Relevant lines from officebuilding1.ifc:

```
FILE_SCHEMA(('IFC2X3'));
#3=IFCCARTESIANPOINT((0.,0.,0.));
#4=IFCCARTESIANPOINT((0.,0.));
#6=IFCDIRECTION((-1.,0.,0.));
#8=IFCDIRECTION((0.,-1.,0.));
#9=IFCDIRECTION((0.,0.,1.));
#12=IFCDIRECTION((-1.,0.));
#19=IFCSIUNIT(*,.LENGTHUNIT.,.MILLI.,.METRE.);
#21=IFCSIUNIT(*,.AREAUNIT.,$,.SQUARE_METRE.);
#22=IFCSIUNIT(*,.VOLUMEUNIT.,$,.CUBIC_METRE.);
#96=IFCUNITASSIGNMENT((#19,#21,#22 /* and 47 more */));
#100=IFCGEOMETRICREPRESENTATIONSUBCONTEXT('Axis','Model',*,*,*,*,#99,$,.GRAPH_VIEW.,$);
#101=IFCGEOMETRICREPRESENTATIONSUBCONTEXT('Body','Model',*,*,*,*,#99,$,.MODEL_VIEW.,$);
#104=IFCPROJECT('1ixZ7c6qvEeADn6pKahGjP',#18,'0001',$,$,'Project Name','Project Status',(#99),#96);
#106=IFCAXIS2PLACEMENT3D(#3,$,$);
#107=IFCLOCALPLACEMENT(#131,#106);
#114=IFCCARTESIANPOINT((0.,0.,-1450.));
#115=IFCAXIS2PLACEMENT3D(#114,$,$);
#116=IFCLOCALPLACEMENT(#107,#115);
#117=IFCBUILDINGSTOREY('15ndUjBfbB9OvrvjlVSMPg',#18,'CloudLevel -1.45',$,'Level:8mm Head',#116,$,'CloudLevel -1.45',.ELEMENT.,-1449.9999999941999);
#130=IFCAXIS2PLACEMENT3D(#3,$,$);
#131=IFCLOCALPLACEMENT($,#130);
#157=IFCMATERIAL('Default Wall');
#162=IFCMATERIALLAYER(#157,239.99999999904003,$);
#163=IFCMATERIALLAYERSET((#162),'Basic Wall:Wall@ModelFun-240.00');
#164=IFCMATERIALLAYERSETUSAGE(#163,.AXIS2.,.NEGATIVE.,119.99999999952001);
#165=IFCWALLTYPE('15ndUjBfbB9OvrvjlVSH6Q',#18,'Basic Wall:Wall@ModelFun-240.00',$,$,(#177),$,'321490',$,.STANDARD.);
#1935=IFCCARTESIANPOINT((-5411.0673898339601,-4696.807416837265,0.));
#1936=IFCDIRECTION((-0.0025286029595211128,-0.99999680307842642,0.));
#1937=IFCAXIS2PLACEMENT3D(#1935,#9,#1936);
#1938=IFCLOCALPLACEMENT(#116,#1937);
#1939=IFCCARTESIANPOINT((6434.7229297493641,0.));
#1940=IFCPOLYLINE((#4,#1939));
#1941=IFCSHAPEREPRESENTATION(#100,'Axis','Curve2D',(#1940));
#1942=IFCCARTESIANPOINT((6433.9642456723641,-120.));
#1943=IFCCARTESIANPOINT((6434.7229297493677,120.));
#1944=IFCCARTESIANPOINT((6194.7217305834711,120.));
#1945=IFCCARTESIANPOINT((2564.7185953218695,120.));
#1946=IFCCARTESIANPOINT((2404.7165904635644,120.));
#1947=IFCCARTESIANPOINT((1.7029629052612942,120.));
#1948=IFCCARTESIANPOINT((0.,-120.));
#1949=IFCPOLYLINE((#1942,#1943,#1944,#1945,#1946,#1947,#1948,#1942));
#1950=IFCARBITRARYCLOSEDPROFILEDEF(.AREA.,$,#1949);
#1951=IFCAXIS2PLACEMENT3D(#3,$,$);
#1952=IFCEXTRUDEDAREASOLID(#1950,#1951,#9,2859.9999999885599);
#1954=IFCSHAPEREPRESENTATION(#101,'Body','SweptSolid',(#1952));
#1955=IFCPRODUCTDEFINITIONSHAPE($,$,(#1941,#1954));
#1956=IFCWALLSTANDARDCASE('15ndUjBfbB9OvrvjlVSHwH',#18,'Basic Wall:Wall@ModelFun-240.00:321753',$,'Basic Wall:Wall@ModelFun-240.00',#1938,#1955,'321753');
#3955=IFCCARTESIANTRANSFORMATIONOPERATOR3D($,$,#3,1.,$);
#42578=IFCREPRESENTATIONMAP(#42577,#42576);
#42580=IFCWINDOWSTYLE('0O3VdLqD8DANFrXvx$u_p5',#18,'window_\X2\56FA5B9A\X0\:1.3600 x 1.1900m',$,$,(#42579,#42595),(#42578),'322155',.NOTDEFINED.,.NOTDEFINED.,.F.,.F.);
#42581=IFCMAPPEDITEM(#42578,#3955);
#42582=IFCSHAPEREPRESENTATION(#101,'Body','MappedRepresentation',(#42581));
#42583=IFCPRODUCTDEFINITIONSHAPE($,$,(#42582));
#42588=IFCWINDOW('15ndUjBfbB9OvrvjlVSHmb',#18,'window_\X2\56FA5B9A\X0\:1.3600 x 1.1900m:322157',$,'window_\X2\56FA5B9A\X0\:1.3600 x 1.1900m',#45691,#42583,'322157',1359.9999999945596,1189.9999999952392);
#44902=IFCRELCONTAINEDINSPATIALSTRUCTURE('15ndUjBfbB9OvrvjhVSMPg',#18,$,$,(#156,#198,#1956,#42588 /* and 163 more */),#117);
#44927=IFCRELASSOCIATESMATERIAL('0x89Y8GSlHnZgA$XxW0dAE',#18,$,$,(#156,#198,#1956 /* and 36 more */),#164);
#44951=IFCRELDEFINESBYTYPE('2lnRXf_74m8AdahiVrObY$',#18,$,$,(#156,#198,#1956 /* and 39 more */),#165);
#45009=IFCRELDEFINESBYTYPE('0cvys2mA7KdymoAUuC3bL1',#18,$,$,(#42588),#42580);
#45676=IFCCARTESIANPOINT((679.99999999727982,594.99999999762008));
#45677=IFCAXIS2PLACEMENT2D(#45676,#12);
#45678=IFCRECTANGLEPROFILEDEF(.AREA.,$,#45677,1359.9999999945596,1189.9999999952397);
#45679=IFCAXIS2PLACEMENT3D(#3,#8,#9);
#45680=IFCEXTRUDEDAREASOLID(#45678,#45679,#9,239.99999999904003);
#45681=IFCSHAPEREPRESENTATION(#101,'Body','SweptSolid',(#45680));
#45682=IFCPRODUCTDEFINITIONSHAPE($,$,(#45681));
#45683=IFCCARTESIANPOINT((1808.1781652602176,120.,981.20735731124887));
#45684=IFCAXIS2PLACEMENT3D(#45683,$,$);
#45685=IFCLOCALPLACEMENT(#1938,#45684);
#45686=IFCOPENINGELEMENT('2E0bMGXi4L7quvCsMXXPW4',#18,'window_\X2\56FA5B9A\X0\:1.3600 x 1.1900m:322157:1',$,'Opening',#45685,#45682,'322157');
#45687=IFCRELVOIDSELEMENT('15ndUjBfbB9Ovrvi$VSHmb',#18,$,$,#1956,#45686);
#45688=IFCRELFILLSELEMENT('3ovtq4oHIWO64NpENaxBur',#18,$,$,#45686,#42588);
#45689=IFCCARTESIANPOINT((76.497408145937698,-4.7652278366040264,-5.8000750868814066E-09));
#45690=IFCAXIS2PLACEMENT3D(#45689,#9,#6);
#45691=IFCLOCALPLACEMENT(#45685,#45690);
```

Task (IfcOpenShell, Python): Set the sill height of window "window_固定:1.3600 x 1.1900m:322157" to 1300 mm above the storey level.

```python
import numpy as np
import ifcopenshell
import ifcopenshell.api.geometry
import ifcopenshell.geom
import ifcopenshell.util.element
import ifcopenshell.util.placement
import ifcopenshell.util.shape
import ifcopenshell.util.unit

model = ifcopenshell.open("officebuilding1.ifc")
unit_scale = ifcopenshell.util.unit.calculate_unit_scale(model)

window = model.by_guid("15ndUjBfbB9OvrvjlVSHmb")
opening = window.FillsVoids[0].RelatingOpeningElement
storey = ifcopenshell.util.element.get_container(window, ifc_class="IfcBuildingStorey")
level = ifcopenshell.util.placement.get_local_placement(storey.ObjectPlacement)[2, 3]

# The opening's origin need not be at the sill, so measure its lowest point.
shape = ifcopenshell.geom.create_shape(ifcopenshell.geom.settings(), opening)
bottom = ifcopenshell.util.shape.get_shape_bottom_elevation(shape, shape.geometry) / unit_scale
dz = level + 1300.0 - bottom

shift = np.array([0.0, 0.0, dz])
# The window is placed relative to its opening, so it follows when the opening moves.
matrix = ifcopenshell.util.placement.get_local_placement(opening.ObjectPlacement)
matrix[:3, 3] += shift
ifcopenshell.api.geometry.edit_object_placement(
    model, product=opening, matrix=matrix, is_si=False, should_transform_children=True
)

print(f"moved by {dz * unit_scale:+.3f} m")

model.write("officebuilding1_v2.ifc")
```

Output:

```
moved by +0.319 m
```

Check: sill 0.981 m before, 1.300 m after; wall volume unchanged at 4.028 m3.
